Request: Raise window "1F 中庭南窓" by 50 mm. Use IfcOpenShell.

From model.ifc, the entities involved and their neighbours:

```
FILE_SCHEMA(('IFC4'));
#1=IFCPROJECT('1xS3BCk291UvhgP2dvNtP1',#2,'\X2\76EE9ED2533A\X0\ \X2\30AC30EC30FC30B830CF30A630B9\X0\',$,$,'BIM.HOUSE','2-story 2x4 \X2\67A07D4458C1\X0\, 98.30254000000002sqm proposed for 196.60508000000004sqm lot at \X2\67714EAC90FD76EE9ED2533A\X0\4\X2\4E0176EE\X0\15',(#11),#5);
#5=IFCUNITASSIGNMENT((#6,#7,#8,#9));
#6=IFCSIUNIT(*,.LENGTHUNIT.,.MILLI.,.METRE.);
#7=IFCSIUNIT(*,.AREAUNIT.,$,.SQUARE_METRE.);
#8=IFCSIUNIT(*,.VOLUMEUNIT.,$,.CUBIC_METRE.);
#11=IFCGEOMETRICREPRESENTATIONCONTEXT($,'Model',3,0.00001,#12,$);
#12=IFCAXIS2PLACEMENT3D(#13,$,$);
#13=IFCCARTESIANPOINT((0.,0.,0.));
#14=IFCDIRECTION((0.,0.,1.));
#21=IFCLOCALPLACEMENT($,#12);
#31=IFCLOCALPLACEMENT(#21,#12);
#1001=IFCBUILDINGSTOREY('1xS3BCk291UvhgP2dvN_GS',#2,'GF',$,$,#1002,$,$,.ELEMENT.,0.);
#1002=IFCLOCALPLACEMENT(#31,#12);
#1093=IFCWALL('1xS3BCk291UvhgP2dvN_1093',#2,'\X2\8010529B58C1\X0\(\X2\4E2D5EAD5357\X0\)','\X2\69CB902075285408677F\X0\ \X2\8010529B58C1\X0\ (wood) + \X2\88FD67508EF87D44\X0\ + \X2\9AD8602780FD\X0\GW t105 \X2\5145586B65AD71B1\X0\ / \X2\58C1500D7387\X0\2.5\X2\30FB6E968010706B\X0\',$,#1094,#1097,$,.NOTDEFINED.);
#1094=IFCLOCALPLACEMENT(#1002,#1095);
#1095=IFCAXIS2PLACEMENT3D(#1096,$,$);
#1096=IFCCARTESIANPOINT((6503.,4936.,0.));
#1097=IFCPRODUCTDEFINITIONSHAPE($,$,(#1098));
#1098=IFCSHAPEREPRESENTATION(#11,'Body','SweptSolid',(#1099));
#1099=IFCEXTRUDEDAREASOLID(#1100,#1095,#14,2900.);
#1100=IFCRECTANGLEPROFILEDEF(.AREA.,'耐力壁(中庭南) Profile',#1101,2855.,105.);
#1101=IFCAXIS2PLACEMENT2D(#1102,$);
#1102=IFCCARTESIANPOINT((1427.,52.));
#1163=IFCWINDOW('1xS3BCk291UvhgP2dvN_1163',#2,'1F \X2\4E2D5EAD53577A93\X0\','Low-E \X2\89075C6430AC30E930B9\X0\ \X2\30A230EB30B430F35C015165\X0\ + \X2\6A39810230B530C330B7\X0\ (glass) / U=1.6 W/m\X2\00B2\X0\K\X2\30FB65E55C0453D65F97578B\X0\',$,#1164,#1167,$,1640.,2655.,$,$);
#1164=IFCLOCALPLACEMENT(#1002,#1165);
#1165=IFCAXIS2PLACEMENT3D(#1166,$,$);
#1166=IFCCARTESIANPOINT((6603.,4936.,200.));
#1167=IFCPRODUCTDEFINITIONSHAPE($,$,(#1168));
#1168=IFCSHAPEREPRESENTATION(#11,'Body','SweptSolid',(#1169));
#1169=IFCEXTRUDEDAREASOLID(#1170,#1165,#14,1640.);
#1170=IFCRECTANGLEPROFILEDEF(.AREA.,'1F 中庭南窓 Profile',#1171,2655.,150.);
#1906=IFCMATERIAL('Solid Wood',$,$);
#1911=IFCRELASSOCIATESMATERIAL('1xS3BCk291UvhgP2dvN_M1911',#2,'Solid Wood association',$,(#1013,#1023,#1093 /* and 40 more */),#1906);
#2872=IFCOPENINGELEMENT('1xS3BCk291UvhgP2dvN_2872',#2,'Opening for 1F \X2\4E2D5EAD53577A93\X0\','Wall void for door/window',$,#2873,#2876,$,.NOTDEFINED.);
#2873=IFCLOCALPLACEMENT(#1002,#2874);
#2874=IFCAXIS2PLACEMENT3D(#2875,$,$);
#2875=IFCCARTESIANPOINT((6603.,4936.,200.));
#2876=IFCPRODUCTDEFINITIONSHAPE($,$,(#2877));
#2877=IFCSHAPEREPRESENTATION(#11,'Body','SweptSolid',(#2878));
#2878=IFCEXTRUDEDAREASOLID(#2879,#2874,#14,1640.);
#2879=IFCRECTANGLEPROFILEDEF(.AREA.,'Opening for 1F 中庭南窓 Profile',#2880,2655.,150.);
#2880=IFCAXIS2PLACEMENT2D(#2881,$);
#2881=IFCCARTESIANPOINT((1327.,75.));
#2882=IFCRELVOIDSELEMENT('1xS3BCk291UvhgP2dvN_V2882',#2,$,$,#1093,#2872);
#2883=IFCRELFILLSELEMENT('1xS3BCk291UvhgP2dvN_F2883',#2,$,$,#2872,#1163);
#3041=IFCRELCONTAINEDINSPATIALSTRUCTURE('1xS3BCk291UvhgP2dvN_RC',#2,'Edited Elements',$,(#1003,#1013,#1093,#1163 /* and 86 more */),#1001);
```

```python
import numpy as np
import ifcopenshell
import ifcopenshell.api.geometry
import ifcopenshell.util.placement
import ifcopenshell.util.unit

model = ifcopenshell.open("model.ifc")
unit_scale = ifcopenshell.util.unit.calculate_unit_scale(model)

window = model.by_guid("1xS3BCk291UvhgP2dvN_1163")
opening = window.FillsVoids[0].RelatingOpeningElement
dz = 0.05 / unit_scale

shift = np.array([0.0, 0.0, dz])
# The window is not placed relative to its opening, so move both.
for product in (opening, window):
    matrix = ifcopenshell.util.placement.get_local_placement(product.ObjectPlacement)
    matrix[:3, 3] += shift
    ifcopenshell.api.geometry.edit_object_placement(model, product=product, matrix=matrix, is_si=False)

print(f"moved by {dz * unit_scale:+.3f} m")

model.write("model_v2.ifc")
```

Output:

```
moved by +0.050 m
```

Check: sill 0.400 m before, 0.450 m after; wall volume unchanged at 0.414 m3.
